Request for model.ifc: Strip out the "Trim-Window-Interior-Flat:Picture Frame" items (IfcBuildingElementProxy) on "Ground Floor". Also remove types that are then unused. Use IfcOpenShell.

First a look at what the model holds.

```python
import ifcopenshell
import ifcopenshell.util.element

model = ifcopenshell.open("model.ifc")
print(model.schema)
storey = next(s for s in model.by_type("IfcBuildingStorey") if s.Name == "Ground Floor")
proxies = [e for e in ifcopenshell.util.element.get_decomposition(storey) if e.is_a("IfcBuildingElementProxy")]
seen = {}
for e in proxies:
    element_type = ifcopenshell.util.element.get_type(e)
    name = element_type.Name if element_type not in (None, e) else None
    seen[name] = seen.get(name, 0) + 1
for name, count in sorted(seen.items(), key=str):
    print(count, "x", name)
```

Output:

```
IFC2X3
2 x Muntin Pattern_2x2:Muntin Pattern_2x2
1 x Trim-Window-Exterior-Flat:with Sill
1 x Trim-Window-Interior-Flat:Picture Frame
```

```python
import ifcopenshell
import ifcopenshell.api.root
import ifcopenshell.util.element

model = ifcopenshell.open("model.ifc")

storey = next(s for s in model.by_type("IfcBuildingStorey") if s.Name == "Ground Floor")
proxies = [e for e in ifcopenshell.util.element.get_decomposition(storey) if e.is_a("IfcBuildingElementProxy")]
targets = [e for e in proxies if (t := ifcopenshell.util.element.get_type(e)) not in (None, e) and t.Name == "Trim-Window-Interior-Flat:Picture Frame"]
types = {ifcopenshell.util.element.get_type(e) for e in targets} - {None, *targets}

for e in targets:
    ifcopenshell.api.root.remove_product(model, product=e)
print(len(targets), "removed")

unused = [t for t in types if not ifcopenshell.util.element.get_types(t)]
for t in unused:
    ifcopenshell.api.root.remove_product(model, product=t)
print(len(unused), "unused types removed")

model.write("model_v2.ifc")
```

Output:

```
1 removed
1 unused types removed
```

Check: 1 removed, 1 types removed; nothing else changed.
